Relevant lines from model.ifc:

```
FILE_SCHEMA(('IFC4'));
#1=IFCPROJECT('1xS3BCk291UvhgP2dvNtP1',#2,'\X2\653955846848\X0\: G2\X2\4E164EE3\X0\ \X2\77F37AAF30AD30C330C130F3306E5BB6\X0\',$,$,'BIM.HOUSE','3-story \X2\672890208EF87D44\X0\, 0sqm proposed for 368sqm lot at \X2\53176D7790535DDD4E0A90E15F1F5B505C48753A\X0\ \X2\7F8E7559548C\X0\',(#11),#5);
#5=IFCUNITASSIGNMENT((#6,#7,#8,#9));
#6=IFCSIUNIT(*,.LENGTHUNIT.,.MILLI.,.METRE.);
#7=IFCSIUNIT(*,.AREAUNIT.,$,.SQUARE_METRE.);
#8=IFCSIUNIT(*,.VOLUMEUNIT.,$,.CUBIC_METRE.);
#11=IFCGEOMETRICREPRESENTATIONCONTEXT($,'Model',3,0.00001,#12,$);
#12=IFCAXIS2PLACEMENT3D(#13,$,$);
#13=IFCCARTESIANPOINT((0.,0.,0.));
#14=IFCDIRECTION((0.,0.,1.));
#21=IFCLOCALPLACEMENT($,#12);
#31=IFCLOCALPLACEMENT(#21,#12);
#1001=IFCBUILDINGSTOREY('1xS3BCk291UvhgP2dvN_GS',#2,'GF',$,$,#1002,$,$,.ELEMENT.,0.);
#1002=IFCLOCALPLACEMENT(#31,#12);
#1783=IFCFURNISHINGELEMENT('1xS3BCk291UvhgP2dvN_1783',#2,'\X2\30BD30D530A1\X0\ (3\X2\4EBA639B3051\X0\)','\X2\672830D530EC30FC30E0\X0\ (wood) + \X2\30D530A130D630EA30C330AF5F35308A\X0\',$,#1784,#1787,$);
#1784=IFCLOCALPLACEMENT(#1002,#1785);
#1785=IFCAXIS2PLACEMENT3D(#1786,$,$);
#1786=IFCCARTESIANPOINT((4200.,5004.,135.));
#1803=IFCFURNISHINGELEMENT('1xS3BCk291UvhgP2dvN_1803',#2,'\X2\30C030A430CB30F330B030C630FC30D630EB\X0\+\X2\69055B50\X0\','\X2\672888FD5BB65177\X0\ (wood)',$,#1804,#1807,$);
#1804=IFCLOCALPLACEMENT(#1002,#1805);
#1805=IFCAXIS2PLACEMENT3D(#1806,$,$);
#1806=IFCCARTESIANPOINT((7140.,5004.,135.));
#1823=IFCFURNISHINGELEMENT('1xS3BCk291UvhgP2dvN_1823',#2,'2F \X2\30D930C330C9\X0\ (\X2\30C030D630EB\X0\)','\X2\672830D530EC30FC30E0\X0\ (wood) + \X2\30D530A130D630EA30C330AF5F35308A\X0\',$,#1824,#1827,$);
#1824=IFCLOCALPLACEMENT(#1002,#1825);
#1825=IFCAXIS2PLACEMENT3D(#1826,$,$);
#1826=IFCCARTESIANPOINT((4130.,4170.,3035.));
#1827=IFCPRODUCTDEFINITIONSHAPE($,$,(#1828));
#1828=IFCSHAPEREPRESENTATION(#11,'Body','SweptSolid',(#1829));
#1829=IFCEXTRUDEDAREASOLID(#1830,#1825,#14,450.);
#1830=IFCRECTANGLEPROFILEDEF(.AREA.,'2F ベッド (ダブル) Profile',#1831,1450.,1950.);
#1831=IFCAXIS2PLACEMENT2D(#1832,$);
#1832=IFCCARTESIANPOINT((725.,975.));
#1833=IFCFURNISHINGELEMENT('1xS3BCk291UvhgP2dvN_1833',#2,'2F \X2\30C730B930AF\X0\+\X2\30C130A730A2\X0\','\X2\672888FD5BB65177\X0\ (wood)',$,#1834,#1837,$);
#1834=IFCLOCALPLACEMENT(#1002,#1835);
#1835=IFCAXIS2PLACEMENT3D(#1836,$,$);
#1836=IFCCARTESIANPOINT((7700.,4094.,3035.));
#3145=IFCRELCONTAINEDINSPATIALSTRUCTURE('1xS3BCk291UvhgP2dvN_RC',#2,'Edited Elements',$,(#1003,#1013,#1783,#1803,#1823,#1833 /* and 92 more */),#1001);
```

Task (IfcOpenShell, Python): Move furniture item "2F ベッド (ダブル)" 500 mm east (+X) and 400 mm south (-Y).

```python
import ifcopenshell
import ifcopenshell.api.geometry
import ifcopenshell.util.placement
import ifcopenshell.util.unit

model = ifcopenshell.open("model.ifc")
unit_scale = ifcopenshell.util.unit.calculate_unit_scale(model)

item = model.by_guid("1xS3BCk291UvhgP2dvN_1823")
matrix = ifcopenshell.util.placement.get_local_placement(item.ObjectPlacement)
matrix[0, 3] += 0.5 / unit_scale
matrix[1, 3] -= 0.4 / unit_scale
ifcopenshell.api.geometry.edit_object_placement(model, product=item, matrix=matrix, is_si=False)

print(ifcopenshell.util.placement.get_local_placement(item.ObjectPlacement).round(3) + 0.0)

model.write("model_edited.ifc")
```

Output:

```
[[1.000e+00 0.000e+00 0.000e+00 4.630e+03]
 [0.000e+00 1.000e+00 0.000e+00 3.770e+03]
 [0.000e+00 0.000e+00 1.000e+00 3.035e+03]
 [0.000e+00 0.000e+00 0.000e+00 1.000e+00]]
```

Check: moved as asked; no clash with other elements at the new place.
